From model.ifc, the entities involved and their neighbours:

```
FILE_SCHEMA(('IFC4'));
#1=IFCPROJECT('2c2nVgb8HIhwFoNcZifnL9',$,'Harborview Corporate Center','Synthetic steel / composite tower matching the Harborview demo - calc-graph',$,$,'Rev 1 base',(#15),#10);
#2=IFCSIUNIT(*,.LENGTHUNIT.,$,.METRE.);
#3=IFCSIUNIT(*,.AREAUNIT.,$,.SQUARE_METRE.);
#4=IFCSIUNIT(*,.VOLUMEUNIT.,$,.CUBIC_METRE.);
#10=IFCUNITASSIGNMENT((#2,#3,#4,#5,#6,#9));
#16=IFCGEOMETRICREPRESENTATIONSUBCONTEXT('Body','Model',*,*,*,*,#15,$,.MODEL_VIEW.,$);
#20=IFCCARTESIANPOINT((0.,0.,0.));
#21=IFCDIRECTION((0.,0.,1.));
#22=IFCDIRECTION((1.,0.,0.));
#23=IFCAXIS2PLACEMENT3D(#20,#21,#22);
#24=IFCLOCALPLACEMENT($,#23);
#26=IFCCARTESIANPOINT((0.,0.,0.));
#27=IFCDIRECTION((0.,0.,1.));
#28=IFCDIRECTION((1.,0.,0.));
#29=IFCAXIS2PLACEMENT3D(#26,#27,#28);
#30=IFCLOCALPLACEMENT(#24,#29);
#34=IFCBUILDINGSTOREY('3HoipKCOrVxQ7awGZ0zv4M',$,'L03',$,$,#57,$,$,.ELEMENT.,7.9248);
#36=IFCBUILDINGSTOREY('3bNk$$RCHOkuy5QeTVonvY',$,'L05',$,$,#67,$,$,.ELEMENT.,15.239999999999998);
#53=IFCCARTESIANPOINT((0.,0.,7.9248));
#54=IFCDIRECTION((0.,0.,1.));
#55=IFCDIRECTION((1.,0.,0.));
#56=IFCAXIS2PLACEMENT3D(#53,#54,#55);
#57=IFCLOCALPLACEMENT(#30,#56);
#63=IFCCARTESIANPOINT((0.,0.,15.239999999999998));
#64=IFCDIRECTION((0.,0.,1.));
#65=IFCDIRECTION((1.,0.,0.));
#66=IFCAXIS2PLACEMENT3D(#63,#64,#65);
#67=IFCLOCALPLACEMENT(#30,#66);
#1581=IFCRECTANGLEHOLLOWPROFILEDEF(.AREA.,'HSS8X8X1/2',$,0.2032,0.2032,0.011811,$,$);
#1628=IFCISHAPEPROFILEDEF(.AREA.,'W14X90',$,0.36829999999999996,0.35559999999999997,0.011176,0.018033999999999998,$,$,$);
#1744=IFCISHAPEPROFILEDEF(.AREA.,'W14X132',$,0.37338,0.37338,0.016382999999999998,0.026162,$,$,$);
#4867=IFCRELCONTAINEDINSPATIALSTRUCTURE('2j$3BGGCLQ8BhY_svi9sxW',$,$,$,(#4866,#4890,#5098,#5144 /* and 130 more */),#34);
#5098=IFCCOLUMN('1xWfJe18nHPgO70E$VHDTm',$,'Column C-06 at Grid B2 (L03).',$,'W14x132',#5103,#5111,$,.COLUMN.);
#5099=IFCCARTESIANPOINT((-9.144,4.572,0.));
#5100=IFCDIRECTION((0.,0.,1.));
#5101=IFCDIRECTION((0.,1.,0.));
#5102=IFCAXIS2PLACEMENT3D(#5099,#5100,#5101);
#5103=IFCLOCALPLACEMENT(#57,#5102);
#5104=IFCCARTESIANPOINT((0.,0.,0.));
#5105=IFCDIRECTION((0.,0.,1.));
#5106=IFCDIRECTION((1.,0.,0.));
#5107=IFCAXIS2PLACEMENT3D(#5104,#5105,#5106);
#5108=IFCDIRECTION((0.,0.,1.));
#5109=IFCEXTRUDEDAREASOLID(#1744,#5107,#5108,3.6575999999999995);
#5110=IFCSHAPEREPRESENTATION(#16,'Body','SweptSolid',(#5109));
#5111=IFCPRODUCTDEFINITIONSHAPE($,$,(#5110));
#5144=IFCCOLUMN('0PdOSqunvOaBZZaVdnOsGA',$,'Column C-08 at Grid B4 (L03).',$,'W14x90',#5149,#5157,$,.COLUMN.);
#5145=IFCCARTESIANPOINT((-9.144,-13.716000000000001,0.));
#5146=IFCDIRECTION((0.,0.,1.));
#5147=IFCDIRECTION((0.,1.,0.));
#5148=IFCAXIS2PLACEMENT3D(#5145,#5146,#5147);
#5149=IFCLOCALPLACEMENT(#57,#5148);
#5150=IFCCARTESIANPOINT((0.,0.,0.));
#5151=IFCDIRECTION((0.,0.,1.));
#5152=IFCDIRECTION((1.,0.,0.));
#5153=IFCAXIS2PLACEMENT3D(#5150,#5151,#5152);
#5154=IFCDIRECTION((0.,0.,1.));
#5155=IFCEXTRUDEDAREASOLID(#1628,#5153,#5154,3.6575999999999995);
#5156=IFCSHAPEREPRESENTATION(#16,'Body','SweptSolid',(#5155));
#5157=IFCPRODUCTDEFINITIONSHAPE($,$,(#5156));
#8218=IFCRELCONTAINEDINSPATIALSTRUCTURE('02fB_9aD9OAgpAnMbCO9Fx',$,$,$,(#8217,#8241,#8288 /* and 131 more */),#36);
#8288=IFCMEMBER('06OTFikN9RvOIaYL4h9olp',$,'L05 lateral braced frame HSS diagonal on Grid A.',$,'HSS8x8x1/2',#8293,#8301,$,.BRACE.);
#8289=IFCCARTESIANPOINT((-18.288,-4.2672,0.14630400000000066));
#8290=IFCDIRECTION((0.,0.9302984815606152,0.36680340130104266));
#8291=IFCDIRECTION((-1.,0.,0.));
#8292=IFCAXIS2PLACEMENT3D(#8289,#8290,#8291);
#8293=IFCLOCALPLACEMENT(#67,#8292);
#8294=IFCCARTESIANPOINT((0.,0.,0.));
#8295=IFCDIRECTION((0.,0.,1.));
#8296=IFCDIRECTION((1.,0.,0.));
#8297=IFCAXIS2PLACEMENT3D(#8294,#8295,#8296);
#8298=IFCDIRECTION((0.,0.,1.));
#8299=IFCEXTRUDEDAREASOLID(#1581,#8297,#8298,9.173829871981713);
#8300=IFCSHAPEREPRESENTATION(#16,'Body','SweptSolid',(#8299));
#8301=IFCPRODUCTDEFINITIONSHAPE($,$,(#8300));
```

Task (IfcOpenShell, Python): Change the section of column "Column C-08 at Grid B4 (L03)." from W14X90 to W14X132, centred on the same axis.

```python
import ifcopenshell
import ifcopenshell.util.element
import ifcopenshell.util.representation

model = ifcopenshell.open("model.ifc")

member = model.by_guid("0PdOSqunvOaBZZaVdnOsGA")
source = next(p for p in model.by_type("IfcIShapeProfileDef") if p.ProfileName == "W14X132")

body = ifcopenshell.util.representation.get_representation(member, "Model", "Body")
solid = body.Items[0]
old_profile = solid.SweptArea

# Copy the section's sizes but keep this member's own profile position.
profile = ifcopenshell.util.element.copy(model, source)
profile.Position = old_profile.Position
solid.SweptArea = profile
if not model.get_total_inverses(old_profile):
    ifcopenshell.util.element.remove_deep2(model, old_profile)

print(solid.SweptArea)

model.write("model_v2.ifc")
```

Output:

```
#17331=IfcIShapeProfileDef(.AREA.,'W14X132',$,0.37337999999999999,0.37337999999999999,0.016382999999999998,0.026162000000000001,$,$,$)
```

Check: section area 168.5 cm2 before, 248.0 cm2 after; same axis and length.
